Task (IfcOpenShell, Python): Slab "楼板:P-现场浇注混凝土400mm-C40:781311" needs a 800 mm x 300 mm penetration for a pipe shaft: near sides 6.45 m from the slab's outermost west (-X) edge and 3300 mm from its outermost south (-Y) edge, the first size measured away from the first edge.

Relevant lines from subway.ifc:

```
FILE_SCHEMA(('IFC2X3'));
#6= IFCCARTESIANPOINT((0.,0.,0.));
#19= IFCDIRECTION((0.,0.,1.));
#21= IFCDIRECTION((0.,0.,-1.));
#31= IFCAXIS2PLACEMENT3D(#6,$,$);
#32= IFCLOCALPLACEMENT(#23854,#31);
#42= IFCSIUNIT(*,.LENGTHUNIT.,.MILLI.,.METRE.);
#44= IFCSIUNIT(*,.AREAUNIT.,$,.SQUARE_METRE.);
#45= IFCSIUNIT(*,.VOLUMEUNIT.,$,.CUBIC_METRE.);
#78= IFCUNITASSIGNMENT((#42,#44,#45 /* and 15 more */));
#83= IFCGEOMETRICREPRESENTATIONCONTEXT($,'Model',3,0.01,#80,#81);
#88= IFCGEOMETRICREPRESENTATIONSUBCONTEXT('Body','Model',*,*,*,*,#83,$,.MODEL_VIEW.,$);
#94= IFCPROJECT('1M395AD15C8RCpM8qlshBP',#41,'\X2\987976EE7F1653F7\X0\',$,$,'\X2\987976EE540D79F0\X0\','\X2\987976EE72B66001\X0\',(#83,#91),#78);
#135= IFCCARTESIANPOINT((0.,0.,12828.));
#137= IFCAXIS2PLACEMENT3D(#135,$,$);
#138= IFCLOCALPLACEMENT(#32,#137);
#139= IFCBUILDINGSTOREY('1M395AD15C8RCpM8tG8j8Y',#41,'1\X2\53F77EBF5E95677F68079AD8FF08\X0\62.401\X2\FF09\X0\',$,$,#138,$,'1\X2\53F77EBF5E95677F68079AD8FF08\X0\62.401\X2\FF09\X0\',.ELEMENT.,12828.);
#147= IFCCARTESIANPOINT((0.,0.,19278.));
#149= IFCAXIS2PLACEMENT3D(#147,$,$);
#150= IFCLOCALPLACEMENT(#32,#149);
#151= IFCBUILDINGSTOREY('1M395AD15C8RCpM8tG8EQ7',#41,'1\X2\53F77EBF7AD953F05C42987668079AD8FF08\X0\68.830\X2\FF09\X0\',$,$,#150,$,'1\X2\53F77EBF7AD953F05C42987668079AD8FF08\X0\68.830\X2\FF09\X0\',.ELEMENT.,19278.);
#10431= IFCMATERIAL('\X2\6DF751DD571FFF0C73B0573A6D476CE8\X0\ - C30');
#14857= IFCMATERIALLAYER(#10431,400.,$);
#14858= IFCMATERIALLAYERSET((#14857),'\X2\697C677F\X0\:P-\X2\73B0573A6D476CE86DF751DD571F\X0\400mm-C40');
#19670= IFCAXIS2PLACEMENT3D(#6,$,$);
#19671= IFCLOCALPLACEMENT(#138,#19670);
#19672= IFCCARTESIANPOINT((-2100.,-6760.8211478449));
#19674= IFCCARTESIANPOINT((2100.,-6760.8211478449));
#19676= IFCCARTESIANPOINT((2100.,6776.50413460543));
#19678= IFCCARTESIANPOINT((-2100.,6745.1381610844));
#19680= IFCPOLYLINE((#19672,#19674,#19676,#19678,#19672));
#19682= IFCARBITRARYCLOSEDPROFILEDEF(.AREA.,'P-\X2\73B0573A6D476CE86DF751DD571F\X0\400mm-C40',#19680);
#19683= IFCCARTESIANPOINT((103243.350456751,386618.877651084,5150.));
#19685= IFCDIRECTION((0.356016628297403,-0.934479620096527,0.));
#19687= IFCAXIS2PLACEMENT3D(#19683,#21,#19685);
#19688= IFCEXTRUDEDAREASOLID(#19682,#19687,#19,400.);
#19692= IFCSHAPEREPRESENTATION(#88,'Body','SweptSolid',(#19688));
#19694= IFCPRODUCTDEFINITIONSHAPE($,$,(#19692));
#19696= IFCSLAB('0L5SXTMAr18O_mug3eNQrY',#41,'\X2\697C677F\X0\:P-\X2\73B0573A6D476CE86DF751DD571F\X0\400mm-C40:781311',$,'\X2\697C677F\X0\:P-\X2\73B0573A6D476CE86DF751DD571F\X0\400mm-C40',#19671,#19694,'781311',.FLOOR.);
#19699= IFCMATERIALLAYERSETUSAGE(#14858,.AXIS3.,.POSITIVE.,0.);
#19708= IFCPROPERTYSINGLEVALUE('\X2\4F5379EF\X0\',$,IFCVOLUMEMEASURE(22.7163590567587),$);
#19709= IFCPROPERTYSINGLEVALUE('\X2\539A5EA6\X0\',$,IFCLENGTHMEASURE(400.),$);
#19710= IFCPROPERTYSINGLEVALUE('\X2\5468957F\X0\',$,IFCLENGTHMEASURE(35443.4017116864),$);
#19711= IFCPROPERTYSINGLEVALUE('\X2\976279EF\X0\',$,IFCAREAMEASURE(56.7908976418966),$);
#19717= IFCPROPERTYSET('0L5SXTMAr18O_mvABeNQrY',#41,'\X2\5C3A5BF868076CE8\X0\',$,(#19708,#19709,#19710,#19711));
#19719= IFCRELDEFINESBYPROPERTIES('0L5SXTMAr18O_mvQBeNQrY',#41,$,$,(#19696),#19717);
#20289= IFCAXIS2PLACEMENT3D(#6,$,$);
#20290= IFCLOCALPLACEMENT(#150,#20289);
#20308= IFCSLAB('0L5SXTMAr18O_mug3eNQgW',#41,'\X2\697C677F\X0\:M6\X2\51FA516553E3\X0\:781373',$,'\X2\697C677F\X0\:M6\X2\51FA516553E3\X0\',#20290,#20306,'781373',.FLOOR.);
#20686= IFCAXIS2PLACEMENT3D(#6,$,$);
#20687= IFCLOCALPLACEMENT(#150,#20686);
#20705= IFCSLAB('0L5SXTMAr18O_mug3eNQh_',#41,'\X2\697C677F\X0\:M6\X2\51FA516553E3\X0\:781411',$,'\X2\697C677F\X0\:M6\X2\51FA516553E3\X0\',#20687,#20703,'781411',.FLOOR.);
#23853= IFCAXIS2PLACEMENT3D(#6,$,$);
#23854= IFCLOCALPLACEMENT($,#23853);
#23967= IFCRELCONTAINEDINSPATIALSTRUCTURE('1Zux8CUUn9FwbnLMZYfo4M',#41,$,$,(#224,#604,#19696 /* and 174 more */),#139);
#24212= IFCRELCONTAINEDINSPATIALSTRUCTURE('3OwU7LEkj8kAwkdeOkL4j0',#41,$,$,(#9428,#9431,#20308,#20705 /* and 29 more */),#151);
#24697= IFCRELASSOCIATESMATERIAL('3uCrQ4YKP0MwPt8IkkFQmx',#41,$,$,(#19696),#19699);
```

```python
import numpy as np
import ifcopenshell
import ifcopenshell.api.feature
import ifcopenshell.api.geometry
import ifcopenshell.api.pset
import ifcopenshell.api.root
import ifcopenshell.geom
import ifcopenshell.util.element
import ifcopenshell.util.placement
import ifcopenshell.util.representation
import ifcopenshell.util.shape
import ifcopenshell.util.unit

model = ifcopenshell.open("subway.ifc")
unit_scale = ifcopenshell.util.unit.calculate_unit_scale(model)
area_scale = ifcopenshell.util.unit.calculate_unit_scale(model, "AREAUNIT")
volume_scale = ifcopenshell.util.unit.calculate_unit_scale(model, "VOLUMEUNIT")
settings = ifcopenshell.geom.settings()


def volume(element):
    """Net volume in cubic metres, openings subtracted."""
    shape = ifcopenshell.geom.create_shape(settings, element)
    return ifcopenshell.util.shape.get_volume(shape.geometry)


slab = model.by_guid("0L5SXTMAr18O_mug3eNQrY")
before = volume(slab)

# Extent in the slab's own axes, in metres. The edges named are its -X and -Y sides.
slab_shape = ifcopenshell.geom.create_shape(settings, slab)
vertices = ifcopenshell.util.shape.get_vertices(slab_shape.geometry)
x_min, y_min, bottom = vertices.min(axis=0)
top = vertices[:, 2].max()

opening = ifcopenshell.api.root.create_entity(model, ifc_class="IfcOpeningElement", name="Pipe shaft opening")
context = ifcopenshell.util.representation.get_context(model, "Model", "Body", "MODEL_VIEW")
width, depth = 0.8, 0.3
outline = [(0.0, 0.0), (width, 0.0), (width, depth), (0.0, depth), (0.0, 0.0)]
# Overshoot both faces by 50 mm so the cut is clean.
shape = ifcopenshell.api.geometry.add_slab_representation(
    model, context=context, depth=top - bottom + 0.1, polyline=outline
)
ifcopenshell.api.geometry.assign_representation(model, product=opening, representation=shape)

matrix = ifcopenshell.util.placement.get_local_placement(slab.ObjectPlacement)
matrix[:, 3] = matrix @ np.append(np.array([x_min + 6.45, y_min + 3.3, bottom - 0.05]) / unit_scale, 1.0)
ifcopenshell.api.geometry.edit_object_placement(model, product=opening, matrix=matrix, is_si=False)
ifcopenshell.api.feature.add_feature(model, feature=opening, element=slab)

after = volume(slab)

# Update the slab's stored quantities.
pset = model.by_id(ifcopenshell.util.element.get_pset(slab, "尺寸标注", should_inherit=False)["id"])
ifcopenshell.api.pset.edit_pset(model, pset=pset, properties={
    "体积": model.create_entity("IfcVolumeMeasure", after / volume_scale),
    "面积": model.create_entity("IfcAreaMeasure", after / (top - bottom) / area_scale),
})

print(f"slab volume {before:.3f} -> {after:.3f} m3")

model.write("subway_updated.ifc")
```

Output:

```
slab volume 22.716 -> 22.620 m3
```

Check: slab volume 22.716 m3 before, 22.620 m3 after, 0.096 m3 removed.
